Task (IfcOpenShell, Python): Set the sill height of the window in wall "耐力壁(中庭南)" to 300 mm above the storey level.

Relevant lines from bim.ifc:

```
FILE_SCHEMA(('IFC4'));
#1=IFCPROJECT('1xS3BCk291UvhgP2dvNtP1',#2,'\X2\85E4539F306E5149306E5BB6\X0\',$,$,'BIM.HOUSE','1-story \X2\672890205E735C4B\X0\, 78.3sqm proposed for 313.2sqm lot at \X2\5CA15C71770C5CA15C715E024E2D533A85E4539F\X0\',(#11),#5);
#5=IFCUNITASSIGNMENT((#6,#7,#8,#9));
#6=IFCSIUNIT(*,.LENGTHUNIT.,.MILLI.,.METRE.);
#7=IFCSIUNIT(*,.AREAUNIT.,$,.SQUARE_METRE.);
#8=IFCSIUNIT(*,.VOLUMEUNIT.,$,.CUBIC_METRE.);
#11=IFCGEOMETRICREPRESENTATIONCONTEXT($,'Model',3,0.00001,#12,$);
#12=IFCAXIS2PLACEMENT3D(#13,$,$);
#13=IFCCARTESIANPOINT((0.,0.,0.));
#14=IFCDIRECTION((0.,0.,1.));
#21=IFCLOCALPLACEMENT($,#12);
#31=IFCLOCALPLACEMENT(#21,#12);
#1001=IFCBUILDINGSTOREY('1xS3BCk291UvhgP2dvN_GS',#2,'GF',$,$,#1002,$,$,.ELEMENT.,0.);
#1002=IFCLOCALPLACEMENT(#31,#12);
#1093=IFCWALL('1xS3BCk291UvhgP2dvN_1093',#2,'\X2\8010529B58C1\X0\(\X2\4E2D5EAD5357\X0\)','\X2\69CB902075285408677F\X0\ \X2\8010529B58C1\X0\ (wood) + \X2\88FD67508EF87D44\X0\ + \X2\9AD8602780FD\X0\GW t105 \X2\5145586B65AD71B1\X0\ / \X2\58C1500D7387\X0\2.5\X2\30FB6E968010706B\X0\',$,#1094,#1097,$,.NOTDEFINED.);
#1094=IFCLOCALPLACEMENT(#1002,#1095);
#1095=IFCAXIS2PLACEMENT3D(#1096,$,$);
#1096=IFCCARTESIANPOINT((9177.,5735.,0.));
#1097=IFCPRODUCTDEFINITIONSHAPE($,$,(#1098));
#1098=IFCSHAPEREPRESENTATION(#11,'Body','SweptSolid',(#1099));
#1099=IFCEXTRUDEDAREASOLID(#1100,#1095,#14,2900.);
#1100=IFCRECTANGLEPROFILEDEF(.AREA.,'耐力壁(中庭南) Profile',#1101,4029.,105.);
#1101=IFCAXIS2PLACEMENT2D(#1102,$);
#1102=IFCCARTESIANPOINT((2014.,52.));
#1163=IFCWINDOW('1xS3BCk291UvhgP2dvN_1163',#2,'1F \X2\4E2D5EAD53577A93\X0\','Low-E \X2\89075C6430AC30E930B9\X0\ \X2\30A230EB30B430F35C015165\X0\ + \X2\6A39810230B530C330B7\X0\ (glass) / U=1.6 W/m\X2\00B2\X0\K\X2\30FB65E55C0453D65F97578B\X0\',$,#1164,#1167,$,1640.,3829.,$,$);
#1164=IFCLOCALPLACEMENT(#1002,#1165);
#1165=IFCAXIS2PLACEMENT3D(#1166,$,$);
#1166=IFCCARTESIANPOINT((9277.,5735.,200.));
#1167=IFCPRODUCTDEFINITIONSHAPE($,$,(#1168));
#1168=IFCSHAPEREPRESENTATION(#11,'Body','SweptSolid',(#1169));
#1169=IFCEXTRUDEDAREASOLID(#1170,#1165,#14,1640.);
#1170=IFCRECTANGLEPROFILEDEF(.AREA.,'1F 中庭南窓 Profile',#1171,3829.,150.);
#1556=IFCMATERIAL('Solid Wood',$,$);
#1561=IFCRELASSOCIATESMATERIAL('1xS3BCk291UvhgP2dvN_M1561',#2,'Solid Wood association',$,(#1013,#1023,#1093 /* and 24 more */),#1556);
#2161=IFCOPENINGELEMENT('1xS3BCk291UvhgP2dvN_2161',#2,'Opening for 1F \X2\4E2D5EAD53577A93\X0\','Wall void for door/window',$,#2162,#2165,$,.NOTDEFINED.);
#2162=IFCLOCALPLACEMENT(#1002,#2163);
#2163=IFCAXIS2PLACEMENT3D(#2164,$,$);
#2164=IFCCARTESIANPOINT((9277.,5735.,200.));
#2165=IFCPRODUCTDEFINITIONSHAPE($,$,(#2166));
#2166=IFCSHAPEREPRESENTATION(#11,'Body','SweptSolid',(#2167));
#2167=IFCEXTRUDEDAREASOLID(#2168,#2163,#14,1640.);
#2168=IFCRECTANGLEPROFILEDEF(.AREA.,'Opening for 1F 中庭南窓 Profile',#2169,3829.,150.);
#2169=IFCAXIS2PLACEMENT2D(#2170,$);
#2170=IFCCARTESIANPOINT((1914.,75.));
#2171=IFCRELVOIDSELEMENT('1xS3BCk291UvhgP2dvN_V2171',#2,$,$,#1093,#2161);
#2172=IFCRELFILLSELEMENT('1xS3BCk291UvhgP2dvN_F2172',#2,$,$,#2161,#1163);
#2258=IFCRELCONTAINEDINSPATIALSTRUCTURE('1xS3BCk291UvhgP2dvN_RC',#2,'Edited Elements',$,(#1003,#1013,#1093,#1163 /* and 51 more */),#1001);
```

```python
import numpy as np
import ifcopenshell
import ifcopenshell.api.geometry
import ifcopenshell.geom
import ifcopenshell.util.element
import ifcopenshell.util.placement
import ifcopenshell.util.shape
import ifcopenshell.util.unit

model = ifcopenshell.open("bim.ifc")
unit_scale = ifcopenshell.util.unit.calculate_unit_scale(model)

window = model.by_guid("1xS3BCk291UvhgP2dvN_1163")
opening = window.FillsVoids[0].RelatingOpeningElement
storey = ifcopenshell.util.element.get_container(window, ifc_class="IfcBuildingStorey")
level = ifcopenshell.util.placement.get_local_placement(storey.ObjectPlacement)[2, 3]

# The opening's origin need not be at the sill, so measure its lowest point.
shape = ifcopenshell.geom.create_shape(ifcopenshell.geom.settings(), opening)
bottom = ifcopenshell.util.shape.get_shape_bottom_elevation(shape, shape.geometry) / unit_scale
dz = level + 300.0 - bottom

shift = np.array([0.0, 0.0, dz])
# The window is not placed relative to its opening, so move both.
for product in (opening, window):
    matrix = ifcopenshell.util.placement.get_local_placement(product.ObjectPlacement)
    matrix[:3, 3] += shift
    ifcopenshell.api.geometry.edit_object_placement(model, product=product, matrix=matrix, is_si=False)

print(f"moved by {dz * unit_scale:+.3f} m")

model.write("bim_v2.ifc")
```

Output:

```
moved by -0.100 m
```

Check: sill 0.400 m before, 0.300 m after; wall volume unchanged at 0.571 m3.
